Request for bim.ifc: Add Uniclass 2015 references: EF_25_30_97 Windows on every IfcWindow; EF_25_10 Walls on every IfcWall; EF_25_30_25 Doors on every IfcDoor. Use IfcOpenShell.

First a look at what the model holds.

```python
import ifcopenshell

model = ifcopenshell.open("bim.ifc")
print(model.schema)
print("classifications:", [c.Name for c in model.by_type("IfcClassification")])
for ifc_class in ("IfcDoor", "IfcRoof", "IfcStair", "IfcWall", "IfcWindow"):
    print(ifc_class, len(model.by_type(ifc_class)))
```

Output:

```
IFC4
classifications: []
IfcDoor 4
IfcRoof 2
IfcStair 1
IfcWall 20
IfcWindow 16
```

```python
import ifcopenshell
import ifcopenshell.api.classification

model = ifcopenshell.open("bim.ifc")

system = ifcopenshell.api.classification.add_classification(model, classification="Uniclass 2015")

codes = {
    "IfcWindow": ("EF_25_30_97", "Windows"),
    "IfcWall": ("EF_25_10", "Walls"),
    "IfcDoor": ("EF_25_30_25", "Doors"),
}
for ifc_class, (code, name) in codes.items():
    products = model.by_type(ifc_class)
    ifcopenshell.api.classification.add_reference(
        model, products=products, classification=system, identification=code, name=name
    )
    print(code, len(products))

model.write("bim_updated.ifc")
```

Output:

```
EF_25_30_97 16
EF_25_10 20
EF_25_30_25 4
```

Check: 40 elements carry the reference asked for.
